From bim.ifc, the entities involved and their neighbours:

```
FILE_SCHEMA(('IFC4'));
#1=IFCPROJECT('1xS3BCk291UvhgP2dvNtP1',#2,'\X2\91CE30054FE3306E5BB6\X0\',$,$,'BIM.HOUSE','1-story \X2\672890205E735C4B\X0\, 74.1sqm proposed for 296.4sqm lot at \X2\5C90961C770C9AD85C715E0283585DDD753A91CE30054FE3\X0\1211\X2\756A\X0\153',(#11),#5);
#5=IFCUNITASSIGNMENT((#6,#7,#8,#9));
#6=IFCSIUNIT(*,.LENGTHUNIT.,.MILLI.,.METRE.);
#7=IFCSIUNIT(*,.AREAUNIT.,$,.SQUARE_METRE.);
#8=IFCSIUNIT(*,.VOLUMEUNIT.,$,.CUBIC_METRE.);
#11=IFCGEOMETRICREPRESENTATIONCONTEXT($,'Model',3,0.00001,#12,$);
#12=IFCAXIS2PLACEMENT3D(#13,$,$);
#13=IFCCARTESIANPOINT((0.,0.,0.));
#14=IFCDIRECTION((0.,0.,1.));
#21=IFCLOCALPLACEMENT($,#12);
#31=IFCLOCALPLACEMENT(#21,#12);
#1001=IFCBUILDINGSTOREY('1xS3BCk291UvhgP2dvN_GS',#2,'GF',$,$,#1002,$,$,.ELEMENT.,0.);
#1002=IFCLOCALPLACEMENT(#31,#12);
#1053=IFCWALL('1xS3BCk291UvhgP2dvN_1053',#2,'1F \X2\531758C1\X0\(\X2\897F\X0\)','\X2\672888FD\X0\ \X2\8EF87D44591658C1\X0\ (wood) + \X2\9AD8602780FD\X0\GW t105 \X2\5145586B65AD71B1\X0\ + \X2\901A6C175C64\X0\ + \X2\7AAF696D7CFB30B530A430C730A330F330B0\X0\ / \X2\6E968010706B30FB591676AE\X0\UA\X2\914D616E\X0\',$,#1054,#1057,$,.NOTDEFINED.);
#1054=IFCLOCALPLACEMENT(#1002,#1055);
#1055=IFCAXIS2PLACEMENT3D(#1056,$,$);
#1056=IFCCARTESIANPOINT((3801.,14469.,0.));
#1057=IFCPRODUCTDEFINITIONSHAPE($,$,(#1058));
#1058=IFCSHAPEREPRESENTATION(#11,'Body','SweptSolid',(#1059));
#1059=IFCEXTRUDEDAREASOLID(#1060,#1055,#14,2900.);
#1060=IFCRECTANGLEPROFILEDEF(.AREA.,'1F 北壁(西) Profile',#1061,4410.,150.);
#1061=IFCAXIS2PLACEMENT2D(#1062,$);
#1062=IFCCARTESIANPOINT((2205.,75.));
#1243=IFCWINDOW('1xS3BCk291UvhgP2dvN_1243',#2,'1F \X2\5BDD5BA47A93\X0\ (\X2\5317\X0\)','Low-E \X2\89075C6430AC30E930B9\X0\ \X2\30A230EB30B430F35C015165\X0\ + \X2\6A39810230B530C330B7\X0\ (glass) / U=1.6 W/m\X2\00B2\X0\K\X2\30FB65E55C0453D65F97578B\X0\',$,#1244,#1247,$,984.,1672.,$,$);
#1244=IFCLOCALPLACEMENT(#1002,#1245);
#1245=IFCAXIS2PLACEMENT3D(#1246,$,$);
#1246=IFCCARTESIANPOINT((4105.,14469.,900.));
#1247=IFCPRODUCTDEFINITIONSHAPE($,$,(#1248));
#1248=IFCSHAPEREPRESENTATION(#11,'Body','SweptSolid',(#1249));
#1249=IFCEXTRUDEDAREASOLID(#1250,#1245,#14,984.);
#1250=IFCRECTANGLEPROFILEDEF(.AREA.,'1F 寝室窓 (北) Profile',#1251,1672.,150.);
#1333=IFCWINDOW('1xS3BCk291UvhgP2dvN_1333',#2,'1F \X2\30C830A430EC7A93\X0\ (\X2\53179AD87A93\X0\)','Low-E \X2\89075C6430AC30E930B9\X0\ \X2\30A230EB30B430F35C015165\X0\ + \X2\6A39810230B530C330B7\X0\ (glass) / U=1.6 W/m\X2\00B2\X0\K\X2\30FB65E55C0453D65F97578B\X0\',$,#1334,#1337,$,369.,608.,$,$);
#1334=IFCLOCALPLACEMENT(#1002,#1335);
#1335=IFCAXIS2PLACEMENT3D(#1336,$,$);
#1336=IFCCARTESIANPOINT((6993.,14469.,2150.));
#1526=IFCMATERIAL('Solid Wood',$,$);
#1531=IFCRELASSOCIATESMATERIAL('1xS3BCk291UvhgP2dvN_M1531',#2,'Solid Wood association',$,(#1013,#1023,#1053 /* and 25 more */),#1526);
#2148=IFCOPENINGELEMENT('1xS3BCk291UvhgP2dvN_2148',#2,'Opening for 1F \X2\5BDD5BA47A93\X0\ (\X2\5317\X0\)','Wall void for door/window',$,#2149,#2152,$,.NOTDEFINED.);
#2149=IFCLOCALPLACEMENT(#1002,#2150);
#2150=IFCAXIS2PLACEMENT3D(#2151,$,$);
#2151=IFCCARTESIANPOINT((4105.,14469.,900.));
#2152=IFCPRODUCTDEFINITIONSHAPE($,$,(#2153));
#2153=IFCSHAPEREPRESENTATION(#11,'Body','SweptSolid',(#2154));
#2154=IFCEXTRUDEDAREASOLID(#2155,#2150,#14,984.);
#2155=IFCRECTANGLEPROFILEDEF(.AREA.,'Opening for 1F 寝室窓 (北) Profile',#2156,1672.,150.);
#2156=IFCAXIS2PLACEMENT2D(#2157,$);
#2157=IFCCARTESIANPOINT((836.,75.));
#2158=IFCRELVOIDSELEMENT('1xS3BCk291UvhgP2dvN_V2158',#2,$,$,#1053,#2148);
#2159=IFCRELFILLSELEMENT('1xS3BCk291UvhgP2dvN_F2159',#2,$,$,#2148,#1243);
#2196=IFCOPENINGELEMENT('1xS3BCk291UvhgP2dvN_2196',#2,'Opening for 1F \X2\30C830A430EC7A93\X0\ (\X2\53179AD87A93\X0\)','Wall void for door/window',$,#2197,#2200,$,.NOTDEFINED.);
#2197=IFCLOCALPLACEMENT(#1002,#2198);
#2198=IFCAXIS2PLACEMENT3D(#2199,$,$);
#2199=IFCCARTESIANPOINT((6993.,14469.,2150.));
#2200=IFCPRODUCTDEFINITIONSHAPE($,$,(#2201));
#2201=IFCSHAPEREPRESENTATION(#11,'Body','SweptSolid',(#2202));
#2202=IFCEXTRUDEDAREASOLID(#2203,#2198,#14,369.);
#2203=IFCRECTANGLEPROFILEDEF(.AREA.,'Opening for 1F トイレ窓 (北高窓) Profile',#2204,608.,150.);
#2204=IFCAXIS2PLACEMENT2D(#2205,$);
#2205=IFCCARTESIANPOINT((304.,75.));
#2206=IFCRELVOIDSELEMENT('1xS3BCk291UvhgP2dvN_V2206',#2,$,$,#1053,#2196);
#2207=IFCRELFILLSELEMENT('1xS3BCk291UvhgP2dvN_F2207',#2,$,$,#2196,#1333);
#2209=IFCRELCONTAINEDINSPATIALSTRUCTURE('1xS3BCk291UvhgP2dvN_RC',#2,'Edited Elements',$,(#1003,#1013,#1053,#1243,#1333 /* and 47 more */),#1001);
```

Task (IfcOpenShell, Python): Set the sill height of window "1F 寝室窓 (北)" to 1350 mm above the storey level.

```python
import numpy as np
import ifcopenshell
import ifcopenshell.api.geometry
import ifcopenshell.geom
import ifcopenshell.util.element
import ifcopenshell.util.placement
import ifcopenshell.util.shape
import ifcopenshell.util.unit

model = ifcopenshell.open("bim.ifc")
unit_scale = ifcopenshell.util.unit.calculate_unit_scale(model)

window = model.by_id(1243)
opening = window.FillsVoids[0].RelatingOpeningElement
storey = ifcopenshell.util.element.get_container(window, ifc_class="IfcBuildingStorey")
level = ifcopenshell.util.placement.get_local_placement(storey.ObjectPlacement)[2, 3]

# The opening's origin need not be at the sill, so measure its lowest point.
shape = ifcopenshell.geom.create_shape(ifcopenshell.geom.settings(), opening)
bottom = ifcopenshell.util.shape.get_shape_bottom_elevation(shape, shape.geometry) / unit_scale
dz = level + 1.35 / unit_scale - bottom

shift = np.array([0.0, 0.0, dz])
# The window is not placed relative to its opening, so move both.
for product in (opening, window):
    matrix = ifcopenshell.util.placement.get_local_placement(product.ObjectPlacement)
    matrix[:3, 3] += shift
    ifcopenshell.api.geometry.edit_object_placement(model, product=product, matrix=matrix, is_si=False)

print(f"moved by {dz * unit_scale:+.3f} m")

model.write("bim-out.ifc")
```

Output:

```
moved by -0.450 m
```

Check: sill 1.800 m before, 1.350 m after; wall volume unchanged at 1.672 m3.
